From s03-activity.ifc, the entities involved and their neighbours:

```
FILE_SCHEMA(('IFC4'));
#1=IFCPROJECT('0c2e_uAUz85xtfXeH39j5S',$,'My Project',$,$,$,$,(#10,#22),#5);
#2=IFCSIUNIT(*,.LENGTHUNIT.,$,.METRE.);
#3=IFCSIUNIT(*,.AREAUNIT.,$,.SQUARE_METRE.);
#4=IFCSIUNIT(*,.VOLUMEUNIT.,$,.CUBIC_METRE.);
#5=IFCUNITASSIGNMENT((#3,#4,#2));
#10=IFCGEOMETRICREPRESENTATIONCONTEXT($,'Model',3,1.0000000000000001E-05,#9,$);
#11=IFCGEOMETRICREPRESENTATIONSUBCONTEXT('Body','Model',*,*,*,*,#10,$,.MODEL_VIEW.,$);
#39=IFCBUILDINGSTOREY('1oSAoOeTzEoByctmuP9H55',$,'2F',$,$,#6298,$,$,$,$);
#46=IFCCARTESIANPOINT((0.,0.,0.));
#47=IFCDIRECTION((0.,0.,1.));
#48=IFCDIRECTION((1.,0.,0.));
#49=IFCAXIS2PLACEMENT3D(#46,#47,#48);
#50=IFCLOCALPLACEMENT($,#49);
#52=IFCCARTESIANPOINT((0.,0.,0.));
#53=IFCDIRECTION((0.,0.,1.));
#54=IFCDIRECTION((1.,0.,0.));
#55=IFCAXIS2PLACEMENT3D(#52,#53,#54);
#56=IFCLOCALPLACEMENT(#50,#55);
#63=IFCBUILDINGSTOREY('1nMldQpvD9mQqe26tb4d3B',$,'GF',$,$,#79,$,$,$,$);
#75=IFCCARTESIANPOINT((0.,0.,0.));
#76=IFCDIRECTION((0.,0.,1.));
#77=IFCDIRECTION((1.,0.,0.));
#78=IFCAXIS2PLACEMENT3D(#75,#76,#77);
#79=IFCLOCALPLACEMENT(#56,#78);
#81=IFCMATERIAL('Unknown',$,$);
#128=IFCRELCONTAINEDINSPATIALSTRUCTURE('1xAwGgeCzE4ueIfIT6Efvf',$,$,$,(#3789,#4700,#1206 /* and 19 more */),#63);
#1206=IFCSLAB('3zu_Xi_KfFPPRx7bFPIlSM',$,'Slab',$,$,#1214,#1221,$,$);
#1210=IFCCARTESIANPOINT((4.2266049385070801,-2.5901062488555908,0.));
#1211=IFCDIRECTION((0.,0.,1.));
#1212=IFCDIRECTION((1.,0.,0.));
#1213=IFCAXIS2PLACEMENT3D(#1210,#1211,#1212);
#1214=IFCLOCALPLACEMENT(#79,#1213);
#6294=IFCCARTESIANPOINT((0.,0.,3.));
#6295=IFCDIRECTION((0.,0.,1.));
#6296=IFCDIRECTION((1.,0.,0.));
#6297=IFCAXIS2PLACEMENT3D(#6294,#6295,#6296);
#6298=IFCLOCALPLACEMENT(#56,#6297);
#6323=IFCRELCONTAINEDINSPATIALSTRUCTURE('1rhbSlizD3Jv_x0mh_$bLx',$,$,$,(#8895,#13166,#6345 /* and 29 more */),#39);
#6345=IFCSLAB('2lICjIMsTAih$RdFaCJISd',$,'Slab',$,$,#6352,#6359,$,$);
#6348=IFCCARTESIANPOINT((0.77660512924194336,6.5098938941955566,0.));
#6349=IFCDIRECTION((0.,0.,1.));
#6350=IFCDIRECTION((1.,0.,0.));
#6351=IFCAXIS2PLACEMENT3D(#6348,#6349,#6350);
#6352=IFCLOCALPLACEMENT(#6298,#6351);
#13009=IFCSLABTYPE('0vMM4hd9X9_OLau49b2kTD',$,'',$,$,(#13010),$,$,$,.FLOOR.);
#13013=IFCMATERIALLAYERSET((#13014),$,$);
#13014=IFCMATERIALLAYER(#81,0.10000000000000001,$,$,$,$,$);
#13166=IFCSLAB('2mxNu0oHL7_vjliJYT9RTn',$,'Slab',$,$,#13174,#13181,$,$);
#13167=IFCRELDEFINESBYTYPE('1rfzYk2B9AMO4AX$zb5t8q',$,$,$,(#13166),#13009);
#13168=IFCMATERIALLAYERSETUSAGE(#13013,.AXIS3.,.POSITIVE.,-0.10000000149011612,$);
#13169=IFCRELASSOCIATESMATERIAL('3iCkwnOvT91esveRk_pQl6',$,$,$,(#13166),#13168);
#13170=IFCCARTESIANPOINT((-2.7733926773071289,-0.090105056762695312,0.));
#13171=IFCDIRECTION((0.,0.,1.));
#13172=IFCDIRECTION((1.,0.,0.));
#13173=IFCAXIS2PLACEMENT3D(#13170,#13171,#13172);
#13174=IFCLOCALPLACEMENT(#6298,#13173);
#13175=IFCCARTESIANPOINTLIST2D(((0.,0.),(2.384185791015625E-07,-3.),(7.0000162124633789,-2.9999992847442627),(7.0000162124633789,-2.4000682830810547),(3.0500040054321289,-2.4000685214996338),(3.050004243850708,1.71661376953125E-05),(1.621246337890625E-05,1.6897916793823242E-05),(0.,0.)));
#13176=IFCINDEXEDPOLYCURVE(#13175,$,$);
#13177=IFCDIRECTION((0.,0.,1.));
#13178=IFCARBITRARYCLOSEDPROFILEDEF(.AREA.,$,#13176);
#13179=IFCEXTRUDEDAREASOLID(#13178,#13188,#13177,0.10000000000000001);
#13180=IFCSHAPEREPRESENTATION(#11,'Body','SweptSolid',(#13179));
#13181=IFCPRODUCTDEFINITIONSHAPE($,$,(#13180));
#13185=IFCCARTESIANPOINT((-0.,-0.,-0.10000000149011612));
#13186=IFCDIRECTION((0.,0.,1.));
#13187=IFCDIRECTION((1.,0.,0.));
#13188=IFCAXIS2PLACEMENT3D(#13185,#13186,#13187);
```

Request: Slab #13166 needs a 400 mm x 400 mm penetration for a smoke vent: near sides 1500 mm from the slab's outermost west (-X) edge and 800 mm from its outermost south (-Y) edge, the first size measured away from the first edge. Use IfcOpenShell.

```python
import numpy as np
import ifcopenshell
import ifcopenshell.api.feature
import ifcopenshell.api.geometry
import ifcopenshell.api.root
import ifcopenshell.geom
import ifcopenshell.util.placement
import ifcopenshell.util.representation
import ifcopenshell.util.shape
import ifcopenshell.util.unit

model = ifcopenshell.open("s03-activity.ifc")
unit_scale = ifcopenshell.util.unit.calculate_unit_scale(model)
settings = ifcopenshell.geom.settings()


def volume(element):
    """Net volume in cubic metres, openings subtracted."""
    shape = ifcopenshell.geom.create_shape(settings, element)
    return ifcopenshell.util.shape.get_volume(shape.geometry)


slab = model.by_id(13166)
before = volume(slab)

# Extent in the slab's own axes, in metres. The edges named are its -X and -Y sides.
slab_shape = ifcopenshell.geom.create_shape(settings, slab)
vertices = ifcopenshell.util.shape.get_vertices(slab_shape.geometry)
x_min, y_min, bottom = vertices.min(axis=0)
top = vertices[:, 2].max()

opening = ifcopenshell.api.root.create_entity(model, ifc_class="IfcOpeningElement", name="Smoke vent opening", predefined_type="OPENING")
context = ifcopenshell.util.representation.get_context(model, "Model", "Body", "MODEL_VIEW")
width, depth = 0.4, 0.4
outline = [(0.0, 0.0), (width, 0.0), (width, depth), (0.0, depth), (0.0, 0.0)]
# Overshoot both faces by 50 mm so the cut is clean.
shape = ifcopenshell.api.geometry.add_slab_representation(
    model, context=context, depth=top - bottom + 0.1, polyline=outline
)
ifcopenshell.api.geometry.assign_representation(model, product=opening, representation=shape)

matrix = ifcopenshell.util.placement.get_local_placement(slab.ObjectPlacement)
matrix[:, 3] = matrix @ np.append(np.array([x_min + 1.5, y_min + 0.8, bottom - 0.05]) / unit_scale, 1.0)
ifcopenshell.api.geometry.edit_object_placement(model, product=opening, matrix=matrix, is_si=False)
ifcopenshell.api.feature.add_feature(model, feature=opening, element=slab)

after = volume(slab)

print(f"slab volume {before:.3f} -> {after:.3f} m3")

model.write("s03-activity_rev.ifc")
```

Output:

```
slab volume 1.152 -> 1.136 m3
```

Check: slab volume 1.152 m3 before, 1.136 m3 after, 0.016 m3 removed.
